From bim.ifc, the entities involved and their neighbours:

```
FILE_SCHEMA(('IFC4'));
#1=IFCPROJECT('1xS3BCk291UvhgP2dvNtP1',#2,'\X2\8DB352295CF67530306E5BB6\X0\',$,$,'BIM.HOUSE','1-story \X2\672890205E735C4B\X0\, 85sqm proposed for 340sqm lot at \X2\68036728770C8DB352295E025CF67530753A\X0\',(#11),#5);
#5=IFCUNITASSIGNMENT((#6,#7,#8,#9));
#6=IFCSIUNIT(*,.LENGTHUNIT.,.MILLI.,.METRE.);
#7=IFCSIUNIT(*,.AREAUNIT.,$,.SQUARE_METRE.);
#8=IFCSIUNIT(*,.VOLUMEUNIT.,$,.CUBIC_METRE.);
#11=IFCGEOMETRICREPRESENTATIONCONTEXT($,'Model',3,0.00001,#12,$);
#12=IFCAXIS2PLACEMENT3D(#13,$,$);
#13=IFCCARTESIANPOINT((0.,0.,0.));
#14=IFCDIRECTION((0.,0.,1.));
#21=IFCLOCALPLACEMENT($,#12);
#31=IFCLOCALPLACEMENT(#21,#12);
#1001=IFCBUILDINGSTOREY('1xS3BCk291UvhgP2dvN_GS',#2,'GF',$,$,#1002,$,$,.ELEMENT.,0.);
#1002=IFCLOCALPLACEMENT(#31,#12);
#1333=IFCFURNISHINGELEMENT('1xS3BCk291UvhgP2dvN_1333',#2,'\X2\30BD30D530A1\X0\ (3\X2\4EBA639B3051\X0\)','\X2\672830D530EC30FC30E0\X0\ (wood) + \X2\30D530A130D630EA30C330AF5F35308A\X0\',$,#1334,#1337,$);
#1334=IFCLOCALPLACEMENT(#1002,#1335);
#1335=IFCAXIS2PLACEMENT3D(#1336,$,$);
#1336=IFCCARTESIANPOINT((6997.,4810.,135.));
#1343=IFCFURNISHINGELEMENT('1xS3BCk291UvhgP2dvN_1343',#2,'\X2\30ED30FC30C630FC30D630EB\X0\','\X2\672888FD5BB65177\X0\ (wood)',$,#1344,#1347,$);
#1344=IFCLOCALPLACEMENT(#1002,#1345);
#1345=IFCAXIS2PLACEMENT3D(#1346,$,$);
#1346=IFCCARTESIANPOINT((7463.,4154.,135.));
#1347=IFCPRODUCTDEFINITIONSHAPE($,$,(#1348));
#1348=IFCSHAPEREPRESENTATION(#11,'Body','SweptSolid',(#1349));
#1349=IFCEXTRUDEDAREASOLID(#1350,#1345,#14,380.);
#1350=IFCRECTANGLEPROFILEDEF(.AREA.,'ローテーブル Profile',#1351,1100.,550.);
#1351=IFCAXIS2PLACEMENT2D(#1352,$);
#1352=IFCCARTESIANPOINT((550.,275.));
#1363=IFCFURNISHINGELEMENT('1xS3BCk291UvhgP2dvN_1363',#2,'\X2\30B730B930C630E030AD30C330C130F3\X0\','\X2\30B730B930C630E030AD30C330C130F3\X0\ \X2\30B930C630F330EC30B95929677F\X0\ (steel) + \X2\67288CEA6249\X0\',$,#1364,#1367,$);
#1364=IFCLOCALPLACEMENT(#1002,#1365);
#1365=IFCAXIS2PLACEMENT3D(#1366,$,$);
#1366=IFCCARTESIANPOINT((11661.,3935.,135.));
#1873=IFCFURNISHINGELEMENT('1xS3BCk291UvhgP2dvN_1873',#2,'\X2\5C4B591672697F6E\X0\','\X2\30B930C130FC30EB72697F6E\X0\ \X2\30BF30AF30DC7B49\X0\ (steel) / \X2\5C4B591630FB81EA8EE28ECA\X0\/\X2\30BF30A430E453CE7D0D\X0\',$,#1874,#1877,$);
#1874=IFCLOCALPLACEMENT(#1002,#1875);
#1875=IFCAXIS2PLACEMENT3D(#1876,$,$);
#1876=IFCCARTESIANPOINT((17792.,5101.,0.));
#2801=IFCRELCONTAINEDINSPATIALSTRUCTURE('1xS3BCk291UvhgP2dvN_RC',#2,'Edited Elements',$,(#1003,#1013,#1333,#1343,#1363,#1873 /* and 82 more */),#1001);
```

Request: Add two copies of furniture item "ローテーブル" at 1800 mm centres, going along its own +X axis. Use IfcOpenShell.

```python
import ifcopenshell
import ifcopenshell.api.geometry
import ifcopenshell.api.root
import ifcopenshell.util.element
import ifcopenshell.util.placement
import ifcopenshell.util.unit

model = ifcopenshell.open("bim.ifc")
unit_scale = ifcopenshell.util.unit.calculate_unit_scale(model)


def reuse_history(source, copy):
    """copy_class also copies each property set's owner history, people and application; keep the originals."""
    for rel in copy.IsDefinedBy:
        if rel.is_a("IfcRelDefinesByProperties") and (history := rel.RelatingPropertyDefinition.OwnerHistory):
            rel.RelatingPropertyDefinition.OwnerHistory = source.OwnerHistory
            ifcopenshell.util.element.remove_deep2(model, history)


source = model.by_guid("1xS3BCk291UvhgP2dvN_1343")
base = ifcopenshell.util.placement.get_local_placement(source.ObjectPlacement)
step = base[:3, 0] * 1.8 / unit_scale

for i in range(1, 3):
    copy = ifcopenshell.api.root.copy_class(model, product=source)
    copy.Representation = ifcopenshell.util.element.copy_deep(
        model, source.Representation, exclude=["IfcGeometricRepresentationContext", "IfcRepresentationMap"]
    )
    reuse_history(source, copy)
    matrix = base.copy()
    matrix[:3, 3] += i * step
    print("added at", matrix[:3, 3].round(3) + 0.0)
    ifcopenshell.api.geometry.edit_object_placement(model, product=copy, matrix=matrix, is_si=False)

model.write("bim_edited.ifc")
```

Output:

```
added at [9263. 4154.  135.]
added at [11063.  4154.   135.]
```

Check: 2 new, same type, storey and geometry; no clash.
